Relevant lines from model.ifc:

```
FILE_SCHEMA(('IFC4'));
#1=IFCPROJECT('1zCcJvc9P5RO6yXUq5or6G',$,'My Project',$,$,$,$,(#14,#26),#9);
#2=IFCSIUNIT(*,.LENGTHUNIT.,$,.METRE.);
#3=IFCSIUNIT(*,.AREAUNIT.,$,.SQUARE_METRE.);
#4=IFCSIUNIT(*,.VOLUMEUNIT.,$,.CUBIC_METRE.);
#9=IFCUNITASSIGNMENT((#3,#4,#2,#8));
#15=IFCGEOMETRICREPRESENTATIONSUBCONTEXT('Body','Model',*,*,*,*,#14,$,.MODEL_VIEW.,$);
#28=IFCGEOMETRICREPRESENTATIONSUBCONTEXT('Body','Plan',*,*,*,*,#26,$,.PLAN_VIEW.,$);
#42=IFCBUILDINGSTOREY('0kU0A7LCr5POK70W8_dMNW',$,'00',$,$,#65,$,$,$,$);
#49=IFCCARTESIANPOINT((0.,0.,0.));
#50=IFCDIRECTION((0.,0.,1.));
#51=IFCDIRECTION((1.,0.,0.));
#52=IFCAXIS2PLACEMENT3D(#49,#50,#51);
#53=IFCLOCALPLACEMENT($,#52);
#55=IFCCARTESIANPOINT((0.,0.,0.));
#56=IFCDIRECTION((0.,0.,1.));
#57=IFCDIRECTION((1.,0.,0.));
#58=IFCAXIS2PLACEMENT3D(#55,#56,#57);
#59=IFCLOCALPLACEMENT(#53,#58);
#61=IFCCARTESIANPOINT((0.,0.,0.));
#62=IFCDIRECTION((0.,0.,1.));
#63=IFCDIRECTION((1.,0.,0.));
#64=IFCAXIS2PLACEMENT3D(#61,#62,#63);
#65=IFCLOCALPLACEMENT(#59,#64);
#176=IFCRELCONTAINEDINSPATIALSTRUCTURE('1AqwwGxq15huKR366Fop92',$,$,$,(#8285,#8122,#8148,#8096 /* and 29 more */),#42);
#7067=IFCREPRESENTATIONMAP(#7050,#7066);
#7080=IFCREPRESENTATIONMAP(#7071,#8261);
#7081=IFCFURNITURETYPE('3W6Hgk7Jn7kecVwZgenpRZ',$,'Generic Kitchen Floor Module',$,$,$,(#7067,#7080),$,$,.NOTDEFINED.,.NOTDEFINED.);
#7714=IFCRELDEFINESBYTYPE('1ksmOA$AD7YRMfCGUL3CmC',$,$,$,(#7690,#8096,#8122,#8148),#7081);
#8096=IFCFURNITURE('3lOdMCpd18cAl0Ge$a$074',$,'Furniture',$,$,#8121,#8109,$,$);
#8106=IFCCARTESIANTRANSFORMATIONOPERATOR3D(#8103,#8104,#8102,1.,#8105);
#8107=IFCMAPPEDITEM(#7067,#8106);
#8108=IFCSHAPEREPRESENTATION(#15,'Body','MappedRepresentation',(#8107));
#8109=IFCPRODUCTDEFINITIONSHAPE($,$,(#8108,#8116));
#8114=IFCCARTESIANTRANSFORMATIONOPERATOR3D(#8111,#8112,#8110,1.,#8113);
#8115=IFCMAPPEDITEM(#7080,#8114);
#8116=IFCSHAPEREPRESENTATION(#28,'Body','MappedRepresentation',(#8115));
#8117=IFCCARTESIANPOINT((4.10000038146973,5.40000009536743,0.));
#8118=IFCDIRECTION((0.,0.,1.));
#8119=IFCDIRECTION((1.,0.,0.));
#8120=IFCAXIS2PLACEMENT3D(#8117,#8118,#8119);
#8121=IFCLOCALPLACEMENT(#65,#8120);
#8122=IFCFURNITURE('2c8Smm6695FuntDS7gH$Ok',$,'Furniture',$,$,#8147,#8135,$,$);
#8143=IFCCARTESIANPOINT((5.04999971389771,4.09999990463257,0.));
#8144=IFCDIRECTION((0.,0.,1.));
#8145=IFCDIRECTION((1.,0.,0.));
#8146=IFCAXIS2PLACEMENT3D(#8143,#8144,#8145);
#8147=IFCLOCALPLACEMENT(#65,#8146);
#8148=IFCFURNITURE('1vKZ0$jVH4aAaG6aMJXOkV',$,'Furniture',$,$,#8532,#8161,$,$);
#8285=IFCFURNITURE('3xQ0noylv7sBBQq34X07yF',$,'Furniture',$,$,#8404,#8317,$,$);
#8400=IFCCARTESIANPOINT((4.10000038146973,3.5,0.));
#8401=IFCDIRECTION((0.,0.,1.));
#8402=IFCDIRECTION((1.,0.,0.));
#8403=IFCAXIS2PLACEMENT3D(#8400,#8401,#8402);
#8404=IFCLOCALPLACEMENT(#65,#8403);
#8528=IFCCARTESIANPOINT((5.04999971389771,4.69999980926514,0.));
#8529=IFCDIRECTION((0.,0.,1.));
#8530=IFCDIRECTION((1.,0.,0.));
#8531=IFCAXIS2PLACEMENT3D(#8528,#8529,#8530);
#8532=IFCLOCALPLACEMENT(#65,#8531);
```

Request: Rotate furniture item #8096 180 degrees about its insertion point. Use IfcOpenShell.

```python
import ifcopenshell
import ifcopenshell.api.geometry
import ifcopenshell.util.placement

model = ifcopenshell.open("model.ifc")

item = model.by_guid("3lOdMCpd18cAl0Ge$a$074")
matrix = ifcopenshell.util.placement.get_local_placement(item.ObjectPlacement)
matrix = matrix @ ifcopenshell.util.placement.rotation(180, "Z")
ifcopenshell.api.geometry.edit_object_placement(model, product=item, matrix=matrix, is_si=False)

print(ifcopenshell.util.placement.get_local_placement(item.ObjectPlacement).round(3) + 0.0)

model.write("model_rev.ifc")
```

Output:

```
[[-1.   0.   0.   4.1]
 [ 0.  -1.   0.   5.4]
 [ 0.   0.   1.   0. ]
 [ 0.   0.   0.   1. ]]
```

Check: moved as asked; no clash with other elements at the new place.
